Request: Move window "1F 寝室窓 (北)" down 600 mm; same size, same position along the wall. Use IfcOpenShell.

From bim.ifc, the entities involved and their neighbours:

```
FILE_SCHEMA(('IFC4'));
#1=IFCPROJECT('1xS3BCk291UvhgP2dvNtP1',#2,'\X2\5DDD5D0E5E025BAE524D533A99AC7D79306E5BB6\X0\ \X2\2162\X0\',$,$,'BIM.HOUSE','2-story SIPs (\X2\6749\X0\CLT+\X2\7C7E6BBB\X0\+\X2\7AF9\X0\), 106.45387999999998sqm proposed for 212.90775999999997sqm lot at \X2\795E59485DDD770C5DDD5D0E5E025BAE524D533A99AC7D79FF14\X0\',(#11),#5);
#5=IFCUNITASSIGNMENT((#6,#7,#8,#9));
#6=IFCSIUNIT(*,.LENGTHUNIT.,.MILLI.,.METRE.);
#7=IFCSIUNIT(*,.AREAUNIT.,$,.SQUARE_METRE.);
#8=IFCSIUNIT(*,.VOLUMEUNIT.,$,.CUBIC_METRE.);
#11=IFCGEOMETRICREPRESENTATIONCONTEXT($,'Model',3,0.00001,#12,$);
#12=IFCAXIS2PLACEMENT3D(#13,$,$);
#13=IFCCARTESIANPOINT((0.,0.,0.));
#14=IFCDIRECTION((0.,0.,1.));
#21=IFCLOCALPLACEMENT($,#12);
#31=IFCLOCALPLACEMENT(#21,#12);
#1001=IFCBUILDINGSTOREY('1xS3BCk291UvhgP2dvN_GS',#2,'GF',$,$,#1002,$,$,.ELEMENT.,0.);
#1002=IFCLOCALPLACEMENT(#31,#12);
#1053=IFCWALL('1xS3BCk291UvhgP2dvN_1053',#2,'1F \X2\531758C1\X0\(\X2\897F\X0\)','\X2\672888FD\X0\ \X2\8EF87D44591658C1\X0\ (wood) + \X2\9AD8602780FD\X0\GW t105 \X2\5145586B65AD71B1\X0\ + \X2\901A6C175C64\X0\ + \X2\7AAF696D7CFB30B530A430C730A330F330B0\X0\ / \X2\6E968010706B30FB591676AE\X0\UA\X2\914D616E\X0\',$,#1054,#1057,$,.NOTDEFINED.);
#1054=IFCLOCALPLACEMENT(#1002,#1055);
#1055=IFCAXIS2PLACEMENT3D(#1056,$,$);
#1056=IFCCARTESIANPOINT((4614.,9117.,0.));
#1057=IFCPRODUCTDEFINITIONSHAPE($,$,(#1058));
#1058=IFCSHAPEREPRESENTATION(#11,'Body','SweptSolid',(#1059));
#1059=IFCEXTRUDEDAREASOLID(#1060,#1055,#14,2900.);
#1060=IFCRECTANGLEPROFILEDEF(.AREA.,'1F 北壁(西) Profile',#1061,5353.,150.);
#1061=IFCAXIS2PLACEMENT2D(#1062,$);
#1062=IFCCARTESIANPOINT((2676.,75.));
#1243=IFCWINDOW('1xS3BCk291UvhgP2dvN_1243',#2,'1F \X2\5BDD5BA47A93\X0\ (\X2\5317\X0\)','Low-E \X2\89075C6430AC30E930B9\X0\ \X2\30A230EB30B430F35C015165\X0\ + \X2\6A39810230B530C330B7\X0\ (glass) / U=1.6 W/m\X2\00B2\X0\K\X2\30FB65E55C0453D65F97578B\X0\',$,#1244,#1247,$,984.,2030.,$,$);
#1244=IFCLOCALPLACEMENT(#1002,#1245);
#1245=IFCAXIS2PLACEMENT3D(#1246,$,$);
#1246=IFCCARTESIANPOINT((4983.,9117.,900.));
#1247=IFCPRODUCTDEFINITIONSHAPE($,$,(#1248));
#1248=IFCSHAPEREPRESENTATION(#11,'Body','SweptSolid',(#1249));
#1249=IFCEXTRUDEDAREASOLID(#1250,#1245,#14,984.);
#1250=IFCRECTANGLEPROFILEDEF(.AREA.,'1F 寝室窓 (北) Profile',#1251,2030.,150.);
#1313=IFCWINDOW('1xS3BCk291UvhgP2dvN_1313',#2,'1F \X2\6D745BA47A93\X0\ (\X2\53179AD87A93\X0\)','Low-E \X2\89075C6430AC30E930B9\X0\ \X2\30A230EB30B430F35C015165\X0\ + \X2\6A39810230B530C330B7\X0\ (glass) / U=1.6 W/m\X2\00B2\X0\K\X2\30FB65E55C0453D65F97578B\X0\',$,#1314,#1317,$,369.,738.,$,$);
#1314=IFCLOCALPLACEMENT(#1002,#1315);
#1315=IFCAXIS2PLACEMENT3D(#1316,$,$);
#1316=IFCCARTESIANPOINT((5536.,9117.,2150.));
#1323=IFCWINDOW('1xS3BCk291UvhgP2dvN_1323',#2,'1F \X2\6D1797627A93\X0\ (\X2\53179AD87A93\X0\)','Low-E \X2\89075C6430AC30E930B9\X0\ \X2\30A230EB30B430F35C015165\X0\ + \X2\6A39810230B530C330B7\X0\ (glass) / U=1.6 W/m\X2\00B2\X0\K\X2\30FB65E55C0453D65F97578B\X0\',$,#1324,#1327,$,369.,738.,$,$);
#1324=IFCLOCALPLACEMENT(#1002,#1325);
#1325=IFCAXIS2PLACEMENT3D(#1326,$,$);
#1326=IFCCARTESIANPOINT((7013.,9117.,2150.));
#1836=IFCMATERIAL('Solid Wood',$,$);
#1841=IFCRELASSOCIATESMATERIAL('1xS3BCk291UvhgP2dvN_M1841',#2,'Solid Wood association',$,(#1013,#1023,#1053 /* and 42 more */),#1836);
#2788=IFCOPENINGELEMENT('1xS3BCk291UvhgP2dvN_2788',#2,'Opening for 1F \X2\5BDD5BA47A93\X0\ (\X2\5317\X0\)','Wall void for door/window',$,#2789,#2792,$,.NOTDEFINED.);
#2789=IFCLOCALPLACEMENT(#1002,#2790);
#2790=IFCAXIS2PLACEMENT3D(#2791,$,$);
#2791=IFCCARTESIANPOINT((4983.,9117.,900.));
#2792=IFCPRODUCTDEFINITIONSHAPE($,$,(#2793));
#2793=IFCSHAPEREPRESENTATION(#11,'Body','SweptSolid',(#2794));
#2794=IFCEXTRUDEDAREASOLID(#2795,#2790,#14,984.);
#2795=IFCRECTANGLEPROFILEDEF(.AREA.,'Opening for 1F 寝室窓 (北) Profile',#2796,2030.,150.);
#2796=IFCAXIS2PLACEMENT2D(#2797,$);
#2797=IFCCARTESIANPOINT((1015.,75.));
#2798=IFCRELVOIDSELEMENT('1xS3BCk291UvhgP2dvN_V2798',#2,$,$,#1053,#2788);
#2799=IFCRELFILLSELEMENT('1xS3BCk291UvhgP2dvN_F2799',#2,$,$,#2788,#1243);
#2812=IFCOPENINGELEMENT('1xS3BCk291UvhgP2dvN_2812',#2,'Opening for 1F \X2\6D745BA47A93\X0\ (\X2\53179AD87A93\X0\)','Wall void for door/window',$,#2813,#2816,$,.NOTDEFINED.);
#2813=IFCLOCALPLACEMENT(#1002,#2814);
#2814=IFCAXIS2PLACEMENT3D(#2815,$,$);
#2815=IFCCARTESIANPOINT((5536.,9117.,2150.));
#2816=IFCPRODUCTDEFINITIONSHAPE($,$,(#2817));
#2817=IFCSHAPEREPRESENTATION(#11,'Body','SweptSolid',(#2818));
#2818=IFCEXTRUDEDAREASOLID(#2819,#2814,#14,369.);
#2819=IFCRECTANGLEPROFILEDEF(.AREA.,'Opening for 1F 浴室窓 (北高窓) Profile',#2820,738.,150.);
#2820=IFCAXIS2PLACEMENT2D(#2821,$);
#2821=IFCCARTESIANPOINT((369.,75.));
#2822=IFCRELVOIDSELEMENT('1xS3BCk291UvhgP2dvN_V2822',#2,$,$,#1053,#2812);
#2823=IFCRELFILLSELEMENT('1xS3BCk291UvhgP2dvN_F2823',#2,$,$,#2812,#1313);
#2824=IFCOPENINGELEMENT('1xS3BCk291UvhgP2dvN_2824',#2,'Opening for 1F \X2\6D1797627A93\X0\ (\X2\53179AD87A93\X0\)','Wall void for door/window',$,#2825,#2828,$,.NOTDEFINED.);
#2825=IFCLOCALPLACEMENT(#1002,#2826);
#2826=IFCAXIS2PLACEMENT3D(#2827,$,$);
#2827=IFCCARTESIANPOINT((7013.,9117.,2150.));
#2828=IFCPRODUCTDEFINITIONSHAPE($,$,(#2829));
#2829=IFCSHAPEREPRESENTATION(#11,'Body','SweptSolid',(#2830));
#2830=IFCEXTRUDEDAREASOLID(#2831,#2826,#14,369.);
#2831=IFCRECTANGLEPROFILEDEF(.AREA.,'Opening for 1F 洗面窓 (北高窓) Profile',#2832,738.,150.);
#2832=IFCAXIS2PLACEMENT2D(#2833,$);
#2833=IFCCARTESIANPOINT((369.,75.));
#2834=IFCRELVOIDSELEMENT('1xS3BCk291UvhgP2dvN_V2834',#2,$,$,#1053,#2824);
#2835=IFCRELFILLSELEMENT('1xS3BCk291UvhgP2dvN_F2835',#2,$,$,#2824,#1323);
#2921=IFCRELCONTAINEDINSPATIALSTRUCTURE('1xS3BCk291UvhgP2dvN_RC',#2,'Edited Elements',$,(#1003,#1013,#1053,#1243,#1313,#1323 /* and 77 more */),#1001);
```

```python
import numpy as np
import ifcopenshell
import ifcopenshell.api.geometry
import ifcopenshell.util.placement
import ifcopenshell.util.unit

model = ifcopenshell.open("bim.ifc")
unit_scale = ifcopenshell.util.unit.calculate_unit_scale(model)

window = model.by_guid("1xS3BCk291UvhgP2dvN_1243")
opening = window.FillsVoids[0].RelatingOpeningElement
dz = -600.0

shift = np.array([0.0, 0.0, dz])
# The window is not placed relative to its opening, so move both.
for product in (opening, window):
    matrix = ifcopenshell.util.placement.get_local_placement(product.ObjectPlacement)
    matrix[:3, 3] += shift
    ifcopenshell.api.geometry.edit_object_placement(model, product=product, matrix=matrix, is_si=False)

print(f"moved by {dz * unit_scale:+.3f} m")

model.write("bim_rev.ifc")
```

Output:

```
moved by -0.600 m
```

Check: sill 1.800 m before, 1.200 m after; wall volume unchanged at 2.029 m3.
